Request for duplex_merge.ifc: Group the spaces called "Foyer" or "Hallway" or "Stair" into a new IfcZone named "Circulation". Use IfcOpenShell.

First a look at what the model holds.

```python
import ifcopenshell

model = ifcopenshell.open("duplex_merge.ifc")
print(model.schema)
seen = {}
for space in model.by_type("IfcSpace"):
    seen[space.LongName] = seen.get(space.LongName, 0) + 1
for name, count in sorted(seen.items(), key=str):
    print(count, "x", name)
print("zones:", [z.Name for z in model.by_type("IfcZone")][:20])
```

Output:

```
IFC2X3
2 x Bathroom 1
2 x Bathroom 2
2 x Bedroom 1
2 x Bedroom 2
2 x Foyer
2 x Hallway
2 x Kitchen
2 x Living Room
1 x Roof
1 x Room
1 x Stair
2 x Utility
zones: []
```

```python
import ifcopenshell
import ifcopenshell.api.group
import ifcopenshell.api.root

model = ifcopenshell.open("duplex_merge.ifc")

names = {"Foyer", "Hallway", "Stair"}
spaces = [s for s in model.by_type("IfcSpace") if s.LongName in names]

zone = ifcopenshell.api.root.create_entity(model, ifc_class="IfcZone", name="Circulation")
ifcopenshell.api.group.assign_group(model, products=spaces, group=zone)
print(len(spaces), "spaces in", zone.Name)

model.write("duplex_merge-out.ifc")
```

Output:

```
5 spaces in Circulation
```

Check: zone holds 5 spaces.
